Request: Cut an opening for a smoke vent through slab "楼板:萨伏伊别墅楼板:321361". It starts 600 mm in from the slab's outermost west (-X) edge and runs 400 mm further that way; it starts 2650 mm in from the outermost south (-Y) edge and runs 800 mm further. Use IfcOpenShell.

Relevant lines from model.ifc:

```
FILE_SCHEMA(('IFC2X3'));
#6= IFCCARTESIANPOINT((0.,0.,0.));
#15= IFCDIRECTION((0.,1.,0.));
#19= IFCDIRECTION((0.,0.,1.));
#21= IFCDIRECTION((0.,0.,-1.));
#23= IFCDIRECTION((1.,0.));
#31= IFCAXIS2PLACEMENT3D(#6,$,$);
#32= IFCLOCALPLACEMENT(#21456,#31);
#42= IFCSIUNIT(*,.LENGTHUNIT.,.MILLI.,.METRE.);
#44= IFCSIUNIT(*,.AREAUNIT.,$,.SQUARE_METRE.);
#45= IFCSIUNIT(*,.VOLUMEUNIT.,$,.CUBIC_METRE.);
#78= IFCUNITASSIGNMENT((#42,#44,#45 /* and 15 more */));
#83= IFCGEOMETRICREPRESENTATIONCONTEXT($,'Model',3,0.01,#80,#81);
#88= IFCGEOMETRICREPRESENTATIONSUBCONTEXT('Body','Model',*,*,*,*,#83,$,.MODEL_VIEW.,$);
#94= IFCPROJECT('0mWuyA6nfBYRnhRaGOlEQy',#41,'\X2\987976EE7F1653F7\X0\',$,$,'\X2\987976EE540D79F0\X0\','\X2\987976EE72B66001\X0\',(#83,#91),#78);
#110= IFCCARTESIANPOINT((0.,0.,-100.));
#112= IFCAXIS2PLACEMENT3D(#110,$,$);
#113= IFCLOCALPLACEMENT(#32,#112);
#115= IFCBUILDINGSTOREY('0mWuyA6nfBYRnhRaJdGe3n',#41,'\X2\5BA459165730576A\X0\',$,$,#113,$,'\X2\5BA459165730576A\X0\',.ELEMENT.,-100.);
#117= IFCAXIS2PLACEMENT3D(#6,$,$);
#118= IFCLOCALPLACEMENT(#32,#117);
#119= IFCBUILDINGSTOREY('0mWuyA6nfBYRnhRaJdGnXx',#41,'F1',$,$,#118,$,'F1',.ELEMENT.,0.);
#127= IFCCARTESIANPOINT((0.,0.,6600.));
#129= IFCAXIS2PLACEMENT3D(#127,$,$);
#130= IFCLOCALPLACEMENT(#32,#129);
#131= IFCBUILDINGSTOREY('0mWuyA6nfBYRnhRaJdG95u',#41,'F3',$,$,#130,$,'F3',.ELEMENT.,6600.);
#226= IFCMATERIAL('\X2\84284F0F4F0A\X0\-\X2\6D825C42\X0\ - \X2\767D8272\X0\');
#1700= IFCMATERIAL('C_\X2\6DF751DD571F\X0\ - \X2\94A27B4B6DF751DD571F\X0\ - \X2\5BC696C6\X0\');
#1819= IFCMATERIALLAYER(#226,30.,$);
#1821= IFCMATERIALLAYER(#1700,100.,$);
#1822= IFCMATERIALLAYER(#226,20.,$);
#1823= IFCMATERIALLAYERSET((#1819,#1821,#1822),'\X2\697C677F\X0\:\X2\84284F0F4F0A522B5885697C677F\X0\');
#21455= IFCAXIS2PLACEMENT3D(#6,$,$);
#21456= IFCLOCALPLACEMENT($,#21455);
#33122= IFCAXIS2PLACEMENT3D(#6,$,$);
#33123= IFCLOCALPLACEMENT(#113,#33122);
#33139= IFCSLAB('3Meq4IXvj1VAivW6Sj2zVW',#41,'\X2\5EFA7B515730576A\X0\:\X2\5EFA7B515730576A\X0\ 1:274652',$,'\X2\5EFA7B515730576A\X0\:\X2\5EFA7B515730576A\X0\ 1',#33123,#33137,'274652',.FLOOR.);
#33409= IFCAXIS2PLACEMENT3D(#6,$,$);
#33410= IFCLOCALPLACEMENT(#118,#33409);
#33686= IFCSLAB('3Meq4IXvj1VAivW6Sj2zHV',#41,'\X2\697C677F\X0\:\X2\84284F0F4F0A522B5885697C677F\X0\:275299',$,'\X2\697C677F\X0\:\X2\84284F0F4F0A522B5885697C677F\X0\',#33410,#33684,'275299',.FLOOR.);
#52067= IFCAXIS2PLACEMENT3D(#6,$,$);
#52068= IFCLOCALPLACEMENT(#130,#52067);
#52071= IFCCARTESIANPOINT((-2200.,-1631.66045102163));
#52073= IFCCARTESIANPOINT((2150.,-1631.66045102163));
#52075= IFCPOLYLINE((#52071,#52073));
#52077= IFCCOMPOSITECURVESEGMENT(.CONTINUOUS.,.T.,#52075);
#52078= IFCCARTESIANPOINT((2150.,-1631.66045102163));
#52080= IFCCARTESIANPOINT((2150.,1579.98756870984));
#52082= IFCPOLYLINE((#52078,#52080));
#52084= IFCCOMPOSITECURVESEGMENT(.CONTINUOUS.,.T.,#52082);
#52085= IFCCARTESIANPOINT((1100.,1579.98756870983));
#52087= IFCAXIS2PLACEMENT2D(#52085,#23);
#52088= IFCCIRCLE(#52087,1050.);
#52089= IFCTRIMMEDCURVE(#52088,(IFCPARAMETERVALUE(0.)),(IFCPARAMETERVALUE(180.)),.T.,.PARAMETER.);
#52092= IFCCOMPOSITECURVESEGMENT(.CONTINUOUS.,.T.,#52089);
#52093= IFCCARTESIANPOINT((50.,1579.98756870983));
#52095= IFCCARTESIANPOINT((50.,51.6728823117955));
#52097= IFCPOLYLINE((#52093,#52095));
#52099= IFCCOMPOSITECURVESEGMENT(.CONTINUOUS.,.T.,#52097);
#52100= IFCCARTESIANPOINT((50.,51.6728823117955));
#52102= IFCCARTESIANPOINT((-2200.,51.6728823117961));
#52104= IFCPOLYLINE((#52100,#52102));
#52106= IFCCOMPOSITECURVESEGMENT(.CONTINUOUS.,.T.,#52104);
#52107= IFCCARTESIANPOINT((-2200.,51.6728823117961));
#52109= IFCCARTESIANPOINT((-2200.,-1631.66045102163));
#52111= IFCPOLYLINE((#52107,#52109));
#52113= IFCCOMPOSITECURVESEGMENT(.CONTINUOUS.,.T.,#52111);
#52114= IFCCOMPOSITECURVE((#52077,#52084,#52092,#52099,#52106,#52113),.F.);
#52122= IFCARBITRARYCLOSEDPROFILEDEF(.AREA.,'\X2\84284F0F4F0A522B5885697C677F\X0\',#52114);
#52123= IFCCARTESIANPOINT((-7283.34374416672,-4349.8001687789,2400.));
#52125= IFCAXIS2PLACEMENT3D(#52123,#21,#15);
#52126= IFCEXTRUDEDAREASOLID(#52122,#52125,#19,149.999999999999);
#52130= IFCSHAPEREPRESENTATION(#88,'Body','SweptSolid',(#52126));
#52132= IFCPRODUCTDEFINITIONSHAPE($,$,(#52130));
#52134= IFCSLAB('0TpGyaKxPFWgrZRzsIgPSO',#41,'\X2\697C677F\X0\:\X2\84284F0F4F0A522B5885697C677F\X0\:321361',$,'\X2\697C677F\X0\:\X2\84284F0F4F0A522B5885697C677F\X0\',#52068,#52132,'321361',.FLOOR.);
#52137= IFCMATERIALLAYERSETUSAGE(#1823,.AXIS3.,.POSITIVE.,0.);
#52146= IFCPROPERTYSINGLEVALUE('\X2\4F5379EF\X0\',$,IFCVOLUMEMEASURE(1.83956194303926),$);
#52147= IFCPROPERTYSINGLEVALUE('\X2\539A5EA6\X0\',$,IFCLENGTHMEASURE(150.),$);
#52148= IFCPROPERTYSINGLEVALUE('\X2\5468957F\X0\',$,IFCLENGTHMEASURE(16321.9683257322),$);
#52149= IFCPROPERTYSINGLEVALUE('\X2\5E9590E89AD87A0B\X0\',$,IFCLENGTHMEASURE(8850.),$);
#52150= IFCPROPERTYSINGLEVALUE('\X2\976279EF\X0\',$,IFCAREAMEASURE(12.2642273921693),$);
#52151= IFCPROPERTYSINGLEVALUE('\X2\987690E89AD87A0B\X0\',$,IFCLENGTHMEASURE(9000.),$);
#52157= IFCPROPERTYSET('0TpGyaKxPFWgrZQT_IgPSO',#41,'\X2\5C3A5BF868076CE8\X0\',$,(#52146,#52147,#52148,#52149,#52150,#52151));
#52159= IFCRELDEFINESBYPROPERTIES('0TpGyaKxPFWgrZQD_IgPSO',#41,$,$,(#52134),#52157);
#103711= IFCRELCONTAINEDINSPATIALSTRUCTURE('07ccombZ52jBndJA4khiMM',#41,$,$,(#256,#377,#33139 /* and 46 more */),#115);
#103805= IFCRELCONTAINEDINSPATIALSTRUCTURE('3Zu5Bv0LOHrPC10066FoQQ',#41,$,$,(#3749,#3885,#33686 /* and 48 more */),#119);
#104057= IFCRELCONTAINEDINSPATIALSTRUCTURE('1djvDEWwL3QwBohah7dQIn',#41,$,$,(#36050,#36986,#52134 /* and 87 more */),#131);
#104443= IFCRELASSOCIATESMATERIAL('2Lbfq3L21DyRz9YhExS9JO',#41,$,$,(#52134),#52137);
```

```python
import numpy as np
import ifcopenshell
import ifcopenshell.api.feature
import ifcopenshell.api.geometry
import ifcopenshell.api.pset
import ifcopenshell.api.root
import ifcopenshell.geom
import ifcopenshell.util.element
import ifcopenshell.util.placement
import ifcopenshell.util.representation
import ifcopenshell.util.shape
import ifcopenshell.util.unit

model = ifcopenshell.open("model.ifc")
unit_scale = ifcopenshell.util.unit.calculate_unit_scale(model)
area_scale = ifcopenshell.util.unit.calculate_unit_scale(model, "AREAUNIT")
volume_scale = ifcopenshell.util.unit.calculate_unit_scale(model, "VOLUMEUNIT")
settings = ifcopenshell.geom.settings()


def volume(element):
    """Net volume in cubic metres, openings subtracted."""
    shape = ifcopenshell.geom.create_shape(settings, element)
    return ifcopenshell.util.shape.get_volume(shape.geometry)


slab = model.by_guid("0TpGyaKxPFWgrZRzsIgPSO")
before = volume(slab)

# Extent in the slab's own axes, in metres. The edges named are its -X and -Y sides.
slab_shape = ifcopenshell.geom.create_shape(settings, slab)
vertices = ifcopenshell.util.shape.get_vertices(slab_shape.geometry)
x_min, y_min, bottom = vertices.min(axis=0)
top = vertices[:, 2].max()

opening = ifcopenshell.api.root.create_entity(model, ifc_class="IfcOpeningElement", name="Smoke vent opening")
context = ifcopenshell.util.representation.get_context(model, "Model", "Body", "MODEL_VIEW")
width, depth = 0.4, 0.8
outline = [(0.0, 0.0), (width, 0.0), (width, depth), (0.0, depth), (0.0, 0.0)]
# Overshoot both faces by 50 mm so the cut is clean.
shape = ifcopenshell.api.geometry.add_slab_representation(
    model, context=context, depth=top - bottom + 0.1, polyline=outline
)
ifcopenshell.api.geometry.assign_representation(model, product=opening, representation=shape)

matrix = ifcopenshell.util.placement.get_local_placement(slab.ObjectPlacement)
matrix[:, 3] = matrix @ np.append(np.array([x_min + 0.6, y_min + 2.65, bottom - 0.05]) / unit_scale, 1.0)
ifcopenshell.api.geometry.edit_object_placement(model, product=opening, matrix=matrix, is_si=False)
ifcopenshell.api.feature.add_feature(model, feature=opening, element=slab)

after = volume(slab)

# Update the slab's stored quantities.
pset = model.by_id(ifcopenshell.util.element.get_pset(slab, "尺寸标注", should_inherit=False)["id"])
ifcopenshell.api.pset.edit_pset(model, pset=pset, properties={
    "体积": model.create_entity("IfcVolumeMeasure", after / volume_scale),
    "面积": model.create_entity("IfcAreaMeasure", after / (top - bottom) / area_scale),
})

print(f"slab volume {before:.3f} -> {after:.3f} m3")

model.write("model_updated.ifc")
```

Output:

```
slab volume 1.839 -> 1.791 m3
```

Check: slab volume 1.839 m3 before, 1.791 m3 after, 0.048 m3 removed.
